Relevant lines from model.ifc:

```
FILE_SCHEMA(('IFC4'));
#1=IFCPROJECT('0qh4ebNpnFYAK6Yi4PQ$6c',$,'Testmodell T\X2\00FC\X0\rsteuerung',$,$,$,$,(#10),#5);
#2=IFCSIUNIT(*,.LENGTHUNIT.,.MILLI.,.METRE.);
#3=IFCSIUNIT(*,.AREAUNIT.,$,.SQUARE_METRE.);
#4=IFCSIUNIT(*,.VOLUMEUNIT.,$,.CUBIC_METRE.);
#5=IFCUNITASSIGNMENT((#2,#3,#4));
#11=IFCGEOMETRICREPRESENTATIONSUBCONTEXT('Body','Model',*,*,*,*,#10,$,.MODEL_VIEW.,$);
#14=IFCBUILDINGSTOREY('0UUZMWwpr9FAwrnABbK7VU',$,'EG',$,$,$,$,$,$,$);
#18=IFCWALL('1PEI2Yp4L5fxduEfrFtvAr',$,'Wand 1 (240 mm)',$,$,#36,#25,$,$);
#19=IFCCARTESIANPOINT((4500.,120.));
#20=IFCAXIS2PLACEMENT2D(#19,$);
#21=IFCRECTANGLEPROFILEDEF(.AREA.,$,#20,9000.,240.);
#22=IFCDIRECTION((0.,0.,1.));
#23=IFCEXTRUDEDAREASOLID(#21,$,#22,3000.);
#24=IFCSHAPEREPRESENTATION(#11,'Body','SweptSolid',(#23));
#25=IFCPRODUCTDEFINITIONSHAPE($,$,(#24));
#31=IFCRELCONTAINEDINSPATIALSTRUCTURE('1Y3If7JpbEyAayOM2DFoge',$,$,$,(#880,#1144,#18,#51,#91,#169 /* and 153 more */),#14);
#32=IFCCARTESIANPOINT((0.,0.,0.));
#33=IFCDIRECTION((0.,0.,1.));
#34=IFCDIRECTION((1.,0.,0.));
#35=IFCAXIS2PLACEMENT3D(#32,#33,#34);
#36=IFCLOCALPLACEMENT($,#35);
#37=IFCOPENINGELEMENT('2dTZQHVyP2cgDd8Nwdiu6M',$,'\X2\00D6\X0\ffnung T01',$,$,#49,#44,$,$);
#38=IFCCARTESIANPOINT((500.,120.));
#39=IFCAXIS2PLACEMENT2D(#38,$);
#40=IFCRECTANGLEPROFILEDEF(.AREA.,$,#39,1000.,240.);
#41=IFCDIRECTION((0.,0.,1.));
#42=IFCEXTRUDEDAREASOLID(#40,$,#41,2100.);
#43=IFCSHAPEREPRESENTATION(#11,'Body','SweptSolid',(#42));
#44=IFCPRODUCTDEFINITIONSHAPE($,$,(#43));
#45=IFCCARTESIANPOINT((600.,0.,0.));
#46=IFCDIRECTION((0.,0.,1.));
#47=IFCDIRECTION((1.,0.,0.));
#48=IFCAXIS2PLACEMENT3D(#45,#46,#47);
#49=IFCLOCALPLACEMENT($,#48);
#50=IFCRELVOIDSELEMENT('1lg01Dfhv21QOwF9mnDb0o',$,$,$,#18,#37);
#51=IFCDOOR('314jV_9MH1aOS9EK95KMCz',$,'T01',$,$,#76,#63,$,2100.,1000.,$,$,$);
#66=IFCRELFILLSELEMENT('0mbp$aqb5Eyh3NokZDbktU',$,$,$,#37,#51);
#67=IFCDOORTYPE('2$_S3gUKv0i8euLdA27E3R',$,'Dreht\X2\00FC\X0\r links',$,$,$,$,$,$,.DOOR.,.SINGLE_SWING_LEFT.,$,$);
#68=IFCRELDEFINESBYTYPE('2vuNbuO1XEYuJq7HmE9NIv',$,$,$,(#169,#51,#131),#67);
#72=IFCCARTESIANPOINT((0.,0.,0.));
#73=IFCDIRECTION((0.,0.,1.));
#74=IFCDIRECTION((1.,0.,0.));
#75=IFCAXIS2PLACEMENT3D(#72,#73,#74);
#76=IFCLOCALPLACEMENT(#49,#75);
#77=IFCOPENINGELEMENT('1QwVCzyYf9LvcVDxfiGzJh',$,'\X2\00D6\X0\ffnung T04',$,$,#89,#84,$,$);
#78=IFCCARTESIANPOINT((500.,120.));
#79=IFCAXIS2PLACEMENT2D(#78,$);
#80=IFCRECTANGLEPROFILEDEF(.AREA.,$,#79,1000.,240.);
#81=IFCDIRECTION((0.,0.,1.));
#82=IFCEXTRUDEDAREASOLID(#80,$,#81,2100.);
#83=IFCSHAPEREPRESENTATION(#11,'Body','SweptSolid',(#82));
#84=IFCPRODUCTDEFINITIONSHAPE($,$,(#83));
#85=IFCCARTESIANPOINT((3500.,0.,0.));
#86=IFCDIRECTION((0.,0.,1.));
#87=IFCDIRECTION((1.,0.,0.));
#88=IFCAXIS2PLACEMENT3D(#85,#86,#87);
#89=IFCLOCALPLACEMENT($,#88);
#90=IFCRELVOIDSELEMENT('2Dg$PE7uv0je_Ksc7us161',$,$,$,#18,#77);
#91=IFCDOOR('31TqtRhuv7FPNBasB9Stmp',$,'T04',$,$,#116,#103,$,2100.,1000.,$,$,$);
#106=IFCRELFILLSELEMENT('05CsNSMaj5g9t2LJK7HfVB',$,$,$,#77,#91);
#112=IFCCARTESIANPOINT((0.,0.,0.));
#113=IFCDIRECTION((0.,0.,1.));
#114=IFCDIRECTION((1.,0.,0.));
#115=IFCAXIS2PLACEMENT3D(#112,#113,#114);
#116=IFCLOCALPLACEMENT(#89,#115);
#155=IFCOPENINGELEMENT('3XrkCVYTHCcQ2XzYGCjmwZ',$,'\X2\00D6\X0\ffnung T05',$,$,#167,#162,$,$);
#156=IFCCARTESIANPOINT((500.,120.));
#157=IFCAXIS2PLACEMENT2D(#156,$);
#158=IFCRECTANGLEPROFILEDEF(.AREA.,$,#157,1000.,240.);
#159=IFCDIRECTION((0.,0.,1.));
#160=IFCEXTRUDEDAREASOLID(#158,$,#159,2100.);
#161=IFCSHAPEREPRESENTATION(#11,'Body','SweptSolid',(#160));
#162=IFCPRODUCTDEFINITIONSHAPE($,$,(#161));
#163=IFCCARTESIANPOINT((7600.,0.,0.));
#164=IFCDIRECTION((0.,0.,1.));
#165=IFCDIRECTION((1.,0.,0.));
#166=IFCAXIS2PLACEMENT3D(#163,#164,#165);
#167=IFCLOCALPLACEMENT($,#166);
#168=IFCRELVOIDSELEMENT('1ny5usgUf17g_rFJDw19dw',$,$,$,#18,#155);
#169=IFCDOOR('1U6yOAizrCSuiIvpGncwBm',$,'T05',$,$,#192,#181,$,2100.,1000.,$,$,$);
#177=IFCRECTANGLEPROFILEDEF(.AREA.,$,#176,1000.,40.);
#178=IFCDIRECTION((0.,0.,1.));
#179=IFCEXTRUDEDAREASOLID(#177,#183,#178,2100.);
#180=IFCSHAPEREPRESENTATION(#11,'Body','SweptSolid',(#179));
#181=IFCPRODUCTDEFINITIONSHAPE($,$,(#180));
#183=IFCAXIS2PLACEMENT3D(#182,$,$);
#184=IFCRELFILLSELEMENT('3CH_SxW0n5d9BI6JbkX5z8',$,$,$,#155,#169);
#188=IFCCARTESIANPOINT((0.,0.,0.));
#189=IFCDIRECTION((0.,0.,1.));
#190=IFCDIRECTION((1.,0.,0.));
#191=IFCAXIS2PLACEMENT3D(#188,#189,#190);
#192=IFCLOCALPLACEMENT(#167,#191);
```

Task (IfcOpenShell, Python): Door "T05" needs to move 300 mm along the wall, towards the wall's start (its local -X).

```python
import ifcopenshell
import ifcopenshell.api.geometry
import ifcopenshell.util.placement
import ifcopenshell.util.unit

model = ifcopenshell.open("model.ifc")
unit_scale = ifcopenshell.util.unit.calculate_unit_scale(model)

door = model.by_guid("1U6yOAizrCSuiIvpGncwBm")
opening = door.FillsVoids[0].RelatingOpeningElement
wall = opening.VoidsElements[0].RelatingBuildingElement

wall_matrix = ifcopenshell.util.placement.get_local_placement(wall.ObjectPlacement)
shift = wall_matrix[:3, 0] * -0.3 / unit_scale
before = ifcopenshell.util.placement.get_local_placement(door.ObjectPlacement)[:3, 3].copy()

# The door is placed relative to its opening, so it follows when the opening moves.
matrix = ifcopenshell.util.placement.get_local_placement(opening.ObjectPlacement)
matrix[:3, 3] += shift
ifcopenshell.api.geometry.edit_object_placement(
    model, product=opening, matrix=matrix, is_si=False, should_transform_children=True
)

after = ifcopenshell.util.placement.get_local_placement(door.ObjectPlacement)[:3, 3]
print("door moved by", (after - before).round(3) + 0.0)

model.write("model_edited.ifc")
```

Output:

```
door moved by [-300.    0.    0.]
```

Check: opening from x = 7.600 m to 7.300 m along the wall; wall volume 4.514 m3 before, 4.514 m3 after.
